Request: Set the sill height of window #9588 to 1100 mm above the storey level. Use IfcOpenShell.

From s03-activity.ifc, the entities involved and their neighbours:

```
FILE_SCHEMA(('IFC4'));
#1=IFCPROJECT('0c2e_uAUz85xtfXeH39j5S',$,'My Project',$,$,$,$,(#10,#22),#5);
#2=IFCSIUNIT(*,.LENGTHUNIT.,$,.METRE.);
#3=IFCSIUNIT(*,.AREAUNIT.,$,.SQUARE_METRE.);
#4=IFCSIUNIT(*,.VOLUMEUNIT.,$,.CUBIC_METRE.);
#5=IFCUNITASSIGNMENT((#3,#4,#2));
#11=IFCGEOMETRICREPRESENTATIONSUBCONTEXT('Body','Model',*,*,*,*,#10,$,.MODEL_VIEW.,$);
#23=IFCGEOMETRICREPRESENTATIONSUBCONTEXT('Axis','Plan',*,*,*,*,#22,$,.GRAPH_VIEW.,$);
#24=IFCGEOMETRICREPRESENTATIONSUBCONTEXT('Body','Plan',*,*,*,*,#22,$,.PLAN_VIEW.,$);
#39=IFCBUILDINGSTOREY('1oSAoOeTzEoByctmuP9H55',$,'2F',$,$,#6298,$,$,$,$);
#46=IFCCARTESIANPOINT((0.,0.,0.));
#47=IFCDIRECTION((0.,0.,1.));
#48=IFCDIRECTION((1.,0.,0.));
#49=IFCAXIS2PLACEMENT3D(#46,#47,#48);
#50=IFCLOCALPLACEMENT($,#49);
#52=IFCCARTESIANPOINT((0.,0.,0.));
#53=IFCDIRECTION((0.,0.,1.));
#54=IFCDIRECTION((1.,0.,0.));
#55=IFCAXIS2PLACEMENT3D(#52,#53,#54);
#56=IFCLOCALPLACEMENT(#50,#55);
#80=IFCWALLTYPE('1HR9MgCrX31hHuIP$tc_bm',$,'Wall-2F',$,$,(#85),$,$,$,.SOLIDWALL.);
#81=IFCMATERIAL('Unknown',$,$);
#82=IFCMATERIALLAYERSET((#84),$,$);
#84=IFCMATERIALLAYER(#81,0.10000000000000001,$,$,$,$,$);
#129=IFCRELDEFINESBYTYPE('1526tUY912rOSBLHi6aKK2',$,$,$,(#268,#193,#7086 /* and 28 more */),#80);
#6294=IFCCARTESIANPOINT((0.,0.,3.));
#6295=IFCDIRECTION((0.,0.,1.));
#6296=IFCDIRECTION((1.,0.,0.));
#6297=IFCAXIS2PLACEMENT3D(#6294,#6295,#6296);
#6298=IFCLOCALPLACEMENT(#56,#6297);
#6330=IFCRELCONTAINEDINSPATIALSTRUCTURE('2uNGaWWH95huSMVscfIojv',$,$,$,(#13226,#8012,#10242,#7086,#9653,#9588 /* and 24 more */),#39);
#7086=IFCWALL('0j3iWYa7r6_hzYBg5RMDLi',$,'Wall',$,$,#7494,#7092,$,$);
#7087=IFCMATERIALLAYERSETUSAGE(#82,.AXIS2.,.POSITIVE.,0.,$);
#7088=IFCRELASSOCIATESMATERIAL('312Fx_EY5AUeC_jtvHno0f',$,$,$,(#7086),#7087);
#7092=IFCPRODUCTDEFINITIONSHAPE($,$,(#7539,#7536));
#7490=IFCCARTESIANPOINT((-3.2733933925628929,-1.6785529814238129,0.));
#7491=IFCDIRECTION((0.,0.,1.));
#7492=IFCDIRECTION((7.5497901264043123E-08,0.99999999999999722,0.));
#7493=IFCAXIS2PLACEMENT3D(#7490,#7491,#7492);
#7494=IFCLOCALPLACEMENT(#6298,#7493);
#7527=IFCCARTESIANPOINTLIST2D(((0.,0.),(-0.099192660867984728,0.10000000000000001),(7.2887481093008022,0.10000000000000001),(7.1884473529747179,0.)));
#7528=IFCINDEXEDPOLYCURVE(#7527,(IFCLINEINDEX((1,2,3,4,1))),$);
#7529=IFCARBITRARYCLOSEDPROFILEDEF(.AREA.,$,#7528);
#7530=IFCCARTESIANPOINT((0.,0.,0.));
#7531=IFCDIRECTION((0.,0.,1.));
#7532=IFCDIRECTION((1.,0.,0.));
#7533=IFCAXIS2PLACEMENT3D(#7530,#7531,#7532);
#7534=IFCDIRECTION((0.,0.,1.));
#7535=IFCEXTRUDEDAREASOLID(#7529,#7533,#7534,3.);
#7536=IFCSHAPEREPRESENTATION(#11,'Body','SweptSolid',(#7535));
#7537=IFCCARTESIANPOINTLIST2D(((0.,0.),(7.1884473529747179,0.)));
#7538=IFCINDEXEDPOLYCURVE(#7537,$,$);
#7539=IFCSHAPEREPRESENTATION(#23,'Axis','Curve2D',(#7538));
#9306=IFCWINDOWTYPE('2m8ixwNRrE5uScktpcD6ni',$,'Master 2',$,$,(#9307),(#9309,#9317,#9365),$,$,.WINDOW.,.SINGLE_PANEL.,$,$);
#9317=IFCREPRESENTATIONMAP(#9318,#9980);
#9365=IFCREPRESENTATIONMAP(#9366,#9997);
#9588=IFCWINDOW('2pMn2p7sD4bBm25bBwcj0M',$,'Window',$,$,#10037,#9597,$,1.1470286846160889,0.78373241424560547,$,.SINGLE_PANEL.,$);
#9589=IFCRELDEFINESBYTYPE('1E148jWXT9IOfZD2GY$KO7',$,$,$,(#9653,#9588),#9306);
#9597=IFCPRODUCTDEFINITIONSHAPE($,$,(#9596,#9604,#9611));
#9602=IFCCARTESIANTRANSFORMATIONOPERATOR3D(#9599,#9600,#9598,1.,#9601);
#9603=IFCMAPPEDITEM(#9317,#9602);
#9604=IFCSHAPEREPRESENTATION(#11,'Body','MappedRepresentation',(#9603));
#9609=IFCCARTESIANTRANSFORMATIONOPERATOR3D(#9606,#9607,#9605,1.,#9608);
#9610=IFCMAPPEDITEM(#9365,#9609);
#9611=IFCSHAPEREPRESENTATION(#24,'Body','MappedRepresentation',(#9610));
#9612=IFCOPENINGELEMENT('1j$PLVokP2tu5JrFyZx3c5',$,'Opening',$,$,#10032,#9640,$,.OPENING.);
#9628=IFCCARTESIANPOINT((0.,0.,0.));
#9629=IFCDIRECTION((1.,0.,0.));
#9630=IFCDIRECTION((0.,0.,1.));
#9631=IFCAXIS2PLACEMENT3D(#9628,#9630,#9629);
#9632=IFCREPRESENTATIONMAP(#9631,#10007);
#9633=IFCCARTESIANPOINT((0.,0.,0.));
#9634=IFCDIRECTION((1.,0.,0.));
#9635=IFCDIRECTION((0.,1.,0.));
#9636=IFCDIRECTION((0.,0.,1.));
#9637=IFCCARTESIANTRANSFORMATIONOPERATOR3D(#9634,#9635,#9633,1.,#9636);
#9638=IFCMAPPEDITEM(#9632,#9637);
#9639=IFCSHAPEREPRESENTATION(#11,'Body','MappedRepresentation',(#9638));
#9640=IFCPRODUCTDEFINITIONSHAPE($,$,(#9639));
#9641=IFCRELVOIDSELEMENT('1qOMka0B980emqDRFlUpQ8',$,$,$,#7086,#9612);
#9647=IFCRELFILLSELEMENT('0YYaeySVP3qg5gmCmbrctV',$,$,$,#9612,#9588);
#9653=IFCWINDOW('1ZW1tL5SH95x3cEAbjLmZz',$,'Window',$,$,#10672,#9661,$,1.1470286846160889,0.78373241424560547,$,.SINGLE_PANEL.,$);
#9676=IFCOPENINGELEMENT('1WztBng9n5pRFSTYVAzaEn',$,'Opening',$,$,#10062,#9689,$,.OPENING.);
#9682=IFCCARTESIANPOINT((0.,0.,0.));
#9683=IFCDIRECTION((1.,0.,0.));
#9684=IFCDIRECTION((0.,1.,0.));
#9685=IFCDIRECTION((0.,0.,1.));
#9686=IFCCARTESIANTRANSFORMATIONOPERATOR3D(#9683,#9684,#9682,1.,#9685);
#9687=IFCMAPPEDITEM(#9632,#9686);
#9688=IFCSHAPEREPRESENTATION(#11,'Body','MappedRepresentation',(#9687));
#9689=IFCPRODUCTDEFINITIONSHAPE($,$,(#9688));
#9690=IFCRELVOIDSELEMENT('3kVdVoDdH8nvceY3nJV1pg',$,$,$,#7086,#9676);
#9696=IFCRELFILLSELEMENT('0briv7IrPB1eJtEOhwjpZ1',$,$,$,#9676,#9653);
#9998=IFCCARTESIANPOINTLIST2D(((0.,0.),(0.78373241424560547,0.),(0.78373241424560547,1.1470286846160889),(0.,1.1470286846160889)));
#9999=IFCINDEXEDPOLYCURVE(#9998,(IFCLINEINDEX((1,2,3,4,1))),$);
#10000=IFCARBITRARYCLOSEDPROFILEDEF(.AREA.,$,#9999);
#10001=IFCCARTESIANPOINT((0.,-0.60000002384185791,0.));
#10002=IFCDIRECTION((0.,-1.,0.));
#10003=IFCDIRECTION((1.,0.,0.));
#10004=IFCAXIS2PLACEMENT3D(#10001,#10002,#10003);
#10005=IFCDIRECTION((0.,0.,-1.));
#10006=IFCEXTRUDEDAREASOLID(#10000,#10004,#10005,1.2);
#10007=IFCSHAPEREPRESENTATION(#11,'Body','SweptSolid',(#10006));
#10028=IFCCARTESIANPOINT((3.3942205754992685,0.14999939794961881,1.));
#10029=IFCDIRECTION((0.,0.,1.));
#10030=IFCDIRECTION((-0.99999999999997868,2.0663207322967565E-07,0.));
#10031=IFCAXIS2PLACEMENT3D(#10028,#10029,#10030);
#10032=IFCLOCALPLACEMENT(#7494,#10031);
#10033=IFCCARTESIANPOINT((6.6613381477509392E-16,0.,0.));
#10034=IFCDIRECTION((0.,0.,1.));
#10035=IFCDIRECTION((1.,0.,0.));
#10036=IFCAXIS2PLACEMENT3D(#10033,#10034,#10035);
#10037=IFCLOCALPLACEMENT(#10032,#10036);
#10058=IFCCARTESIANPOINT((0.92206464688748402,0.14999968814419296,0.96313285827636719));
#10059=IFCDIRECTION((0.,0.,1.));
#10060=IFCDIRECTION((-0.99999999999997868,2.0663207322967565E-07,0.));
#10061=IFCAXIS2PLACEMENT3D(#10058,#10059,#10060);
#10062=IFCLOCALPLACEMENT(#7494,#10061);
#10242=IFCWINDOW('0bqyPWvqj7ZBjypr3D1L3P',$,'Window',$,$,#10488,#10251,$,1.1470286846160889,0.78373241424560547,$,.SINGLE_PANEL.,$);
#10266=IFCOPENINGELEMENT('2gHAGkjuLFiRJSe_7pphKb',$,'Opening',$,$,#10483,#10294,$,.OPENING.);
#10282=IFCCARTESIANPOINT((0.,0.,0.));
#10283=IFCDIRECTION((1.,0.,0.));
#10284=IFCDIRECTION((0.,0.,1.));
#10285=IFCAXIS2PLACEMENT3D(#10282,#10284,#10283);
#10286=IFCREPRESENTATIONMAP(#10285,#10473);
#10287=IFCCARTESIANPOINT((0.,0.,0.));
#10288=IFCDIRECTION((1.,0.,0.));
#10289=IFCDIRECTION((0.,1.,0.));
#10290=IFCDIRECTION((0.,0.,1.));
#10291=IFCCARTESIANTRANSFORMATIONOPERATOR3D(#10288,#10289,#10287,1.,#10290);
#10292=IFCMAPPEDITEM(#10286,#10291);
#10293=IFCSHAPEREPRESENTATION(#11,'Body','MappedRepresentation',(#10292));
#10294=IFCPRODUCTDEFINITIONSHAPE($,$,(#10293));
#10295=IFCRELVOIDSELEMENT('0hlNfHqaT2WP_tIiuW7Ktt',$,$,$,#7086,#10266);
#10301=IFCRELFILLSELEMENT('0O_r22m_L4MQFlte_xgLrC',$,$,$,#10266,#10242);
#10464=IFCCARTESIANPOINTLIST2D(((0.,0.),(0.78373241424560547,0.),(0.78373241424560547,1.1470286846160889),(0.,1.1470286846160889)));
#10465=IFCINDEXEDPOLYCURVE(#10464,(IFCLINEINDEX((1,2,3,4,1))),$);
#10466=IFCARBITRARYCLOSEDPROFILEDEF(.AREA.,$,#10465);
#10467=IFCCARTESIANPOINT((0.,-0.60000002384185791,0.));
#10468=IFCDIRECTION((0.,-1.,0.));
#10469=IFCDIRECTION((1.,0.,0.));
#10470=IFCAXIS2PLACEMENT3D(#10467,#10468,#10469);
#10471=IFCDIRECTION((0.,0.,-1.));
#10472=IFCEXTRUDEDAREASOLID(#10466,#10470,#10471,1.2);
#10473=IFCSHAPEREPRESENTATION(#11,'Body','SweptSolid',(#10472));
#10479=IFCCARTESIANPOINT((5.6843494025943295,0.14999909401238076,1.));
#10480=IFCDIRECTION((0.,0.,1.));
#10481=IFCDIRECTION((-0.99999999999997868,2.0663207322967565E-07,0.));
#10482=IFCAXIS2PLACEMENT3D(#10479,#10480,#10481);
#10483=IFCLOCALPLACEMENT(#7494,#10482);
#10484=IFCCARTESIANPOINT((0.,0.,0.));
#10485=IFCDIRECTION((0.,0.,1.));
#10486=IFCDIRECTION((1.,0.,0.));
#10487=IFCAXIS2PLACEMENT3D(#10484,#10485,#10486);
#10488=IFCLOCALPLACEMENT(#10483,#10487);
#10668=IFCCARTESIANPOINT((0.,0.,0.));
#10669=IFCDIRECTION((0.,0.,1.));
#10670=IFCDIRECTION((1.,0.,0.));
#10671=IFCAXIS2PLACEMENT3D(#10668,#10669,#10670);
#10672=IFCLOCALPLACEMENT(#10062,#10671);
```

```python
import numpy as np
import ifcopenshell
import ifcopenshell.api.geometry
import ifcopenshell.geom
import ifcopenshell.util.element
import ifcopenshell.util.placement
import ifcopenshell.util.shape
import ifcopenshell.util.unit

model = ifcopenshell.open("s03-activity.ifc")
unit_scale = ifcopenshell.util.unit.calculate_unit_scale(model)

window = model.by_id(9588)
opening = window.FillsVoids[0].RelatingOpeningElement
storey = ifcopenshell.util.element.get_container(window, ifc_class="IfcBuildingStorey")
level = ifcopenshell.util.placement.get_local_placement(storey.ObjectPlacement)[2, 3]

# The opening's origin need not be at the sill, so measure its lowest point.
shape = ifcopenshell.geom.create_shape(ifcopenshell.geom.settings(), opening)
bottom = ifcopenshell.util.shape.get_shape_bottom_elevation(shape, shape.geometry) / unit_scale
dz = level + 1.1 - bottom

shift = np.array([0.0, 0.0, dz])
# The window is placed relative to its opening, so it follows when the opening moves.
matrix = ifcopenshell.util.placement.get_local_placement(opening.ObjectPlacement)
matrix[:3, 3] += shift
ifcopenshell.api.geometry.edit_object_placement(
    model, product=opening, matrix=matrix, is_si=False, should_transform_children=True
)

print(f"moved by {dz * unit_scale:+.3f} m")

model.write("s03-activity-out.ifc")
```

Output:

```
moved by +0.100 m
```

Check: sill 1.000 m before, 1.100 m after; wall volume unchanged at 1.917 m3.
